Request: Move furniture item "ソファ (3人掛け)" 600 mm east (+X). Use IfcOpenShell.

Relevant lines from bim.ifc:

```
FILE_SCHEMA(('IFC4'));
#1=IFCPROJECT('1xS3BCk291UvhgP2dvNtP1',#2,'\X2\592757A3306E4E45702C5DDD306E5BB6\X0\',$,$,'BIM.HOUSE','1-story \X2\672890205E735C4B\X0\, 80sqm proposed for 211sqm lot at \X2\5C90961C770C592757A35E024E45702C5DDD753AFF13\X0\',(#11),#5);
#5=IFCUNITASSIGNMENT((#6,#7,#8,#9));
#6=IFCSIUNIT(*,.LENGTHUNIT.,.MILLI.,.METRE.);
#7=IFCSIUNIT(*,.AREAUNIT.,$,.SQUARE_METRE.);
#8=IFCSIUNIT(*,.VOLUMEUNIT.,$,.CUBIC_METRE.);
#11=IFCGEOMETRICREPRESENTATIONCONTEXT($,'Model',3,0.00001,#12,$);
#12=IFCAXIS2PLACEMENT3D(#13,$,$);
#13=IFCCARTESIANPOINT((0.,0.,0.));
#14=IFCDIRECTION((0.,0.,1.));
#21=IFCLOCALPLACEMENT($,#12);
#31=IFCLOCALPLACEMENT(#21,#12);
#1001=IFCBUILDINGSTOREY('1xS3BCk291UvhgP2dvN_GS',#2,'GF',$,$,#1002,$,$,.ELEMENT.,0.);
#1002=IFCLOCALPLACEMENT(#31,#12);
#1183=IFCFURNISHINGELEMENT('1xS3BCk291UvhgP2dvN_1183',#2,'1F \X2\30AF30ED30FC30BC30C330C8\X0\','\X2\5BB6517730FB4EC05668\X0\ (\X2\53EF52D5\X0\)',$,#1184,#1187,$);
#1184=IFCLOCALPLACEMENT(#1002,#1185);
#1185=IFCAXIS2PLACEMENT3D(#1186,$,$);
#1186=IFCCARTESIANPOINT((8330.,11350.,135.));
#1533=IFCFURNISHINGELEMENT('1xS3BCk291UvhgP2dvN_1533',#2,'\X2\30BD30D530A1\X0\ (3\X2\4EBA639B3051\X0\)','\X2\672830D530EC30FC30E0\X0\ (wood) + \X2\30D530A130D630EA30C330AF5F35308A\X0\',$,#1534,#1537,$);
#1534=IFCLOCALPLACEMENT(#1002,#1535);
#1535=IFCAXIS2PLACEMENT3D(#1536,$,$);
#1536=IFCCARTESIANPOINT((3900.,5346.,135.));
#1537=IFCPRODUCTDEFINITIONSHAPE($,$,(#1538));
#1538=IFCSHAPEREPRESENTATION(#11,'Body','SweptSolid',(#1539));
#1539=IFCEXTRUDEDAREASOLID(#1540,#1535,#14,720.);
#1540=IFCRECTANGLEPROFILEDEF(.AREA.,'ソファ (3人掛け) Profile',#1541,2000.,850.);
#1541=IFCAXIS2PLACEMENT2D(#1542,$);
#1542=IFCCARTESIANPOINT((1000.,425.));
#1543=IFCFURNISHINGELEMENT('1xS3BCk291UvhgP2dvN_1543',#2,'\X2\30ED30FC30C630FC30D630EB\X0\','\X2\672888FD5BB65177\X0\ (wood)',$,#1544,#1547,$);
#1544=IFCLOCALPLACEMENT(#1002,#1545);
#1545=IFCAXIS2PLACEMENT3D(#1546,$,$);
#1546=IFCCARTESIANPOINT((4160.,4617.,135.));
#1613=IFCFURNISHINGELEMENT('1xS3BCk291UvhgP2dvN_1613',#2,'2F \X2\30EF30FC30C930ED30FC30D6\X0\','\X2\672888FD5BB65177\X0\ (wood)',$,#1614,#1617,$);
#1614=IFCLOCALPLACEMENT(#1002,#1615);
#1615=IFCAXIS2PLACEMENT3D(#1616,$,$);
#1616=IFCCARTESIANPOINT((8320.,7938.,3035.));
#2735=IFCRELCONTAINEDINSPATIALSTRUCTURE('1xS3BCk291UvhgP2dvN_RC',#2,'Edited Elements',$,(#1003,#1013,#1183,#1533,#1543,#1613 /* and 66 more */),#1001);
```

```python
import ifcopenshell
import ifcopenshell.api.geometry
import ifcopenshell.util.placement

model = ifcopenshell.open("bim.ifc")

item = model.by_guid("1xS3BCk291UvhgP2dvN_1533")
matrix = ifcopenshell.util.placement.get_local_placement(item.ObjectPlacement)
matrix[0, 3] += 600.0
ifcopenshell.api.geometry.edit_object_placement(model, product=item, matrix=matrix, is_si=False)

print(ifcopenshell.util.placement.get_local_placement(item.ObjectPlacement).round(3) + 0.0)

model.write("bim_v2.ifc")
```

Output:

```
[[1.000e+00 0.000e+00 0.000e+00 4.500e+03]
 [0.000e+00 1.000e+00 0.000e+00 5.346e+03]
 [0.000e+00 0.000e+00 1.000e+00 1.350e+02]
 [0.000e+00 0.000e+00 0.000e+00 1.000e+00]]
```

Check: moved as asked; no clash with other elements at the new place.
